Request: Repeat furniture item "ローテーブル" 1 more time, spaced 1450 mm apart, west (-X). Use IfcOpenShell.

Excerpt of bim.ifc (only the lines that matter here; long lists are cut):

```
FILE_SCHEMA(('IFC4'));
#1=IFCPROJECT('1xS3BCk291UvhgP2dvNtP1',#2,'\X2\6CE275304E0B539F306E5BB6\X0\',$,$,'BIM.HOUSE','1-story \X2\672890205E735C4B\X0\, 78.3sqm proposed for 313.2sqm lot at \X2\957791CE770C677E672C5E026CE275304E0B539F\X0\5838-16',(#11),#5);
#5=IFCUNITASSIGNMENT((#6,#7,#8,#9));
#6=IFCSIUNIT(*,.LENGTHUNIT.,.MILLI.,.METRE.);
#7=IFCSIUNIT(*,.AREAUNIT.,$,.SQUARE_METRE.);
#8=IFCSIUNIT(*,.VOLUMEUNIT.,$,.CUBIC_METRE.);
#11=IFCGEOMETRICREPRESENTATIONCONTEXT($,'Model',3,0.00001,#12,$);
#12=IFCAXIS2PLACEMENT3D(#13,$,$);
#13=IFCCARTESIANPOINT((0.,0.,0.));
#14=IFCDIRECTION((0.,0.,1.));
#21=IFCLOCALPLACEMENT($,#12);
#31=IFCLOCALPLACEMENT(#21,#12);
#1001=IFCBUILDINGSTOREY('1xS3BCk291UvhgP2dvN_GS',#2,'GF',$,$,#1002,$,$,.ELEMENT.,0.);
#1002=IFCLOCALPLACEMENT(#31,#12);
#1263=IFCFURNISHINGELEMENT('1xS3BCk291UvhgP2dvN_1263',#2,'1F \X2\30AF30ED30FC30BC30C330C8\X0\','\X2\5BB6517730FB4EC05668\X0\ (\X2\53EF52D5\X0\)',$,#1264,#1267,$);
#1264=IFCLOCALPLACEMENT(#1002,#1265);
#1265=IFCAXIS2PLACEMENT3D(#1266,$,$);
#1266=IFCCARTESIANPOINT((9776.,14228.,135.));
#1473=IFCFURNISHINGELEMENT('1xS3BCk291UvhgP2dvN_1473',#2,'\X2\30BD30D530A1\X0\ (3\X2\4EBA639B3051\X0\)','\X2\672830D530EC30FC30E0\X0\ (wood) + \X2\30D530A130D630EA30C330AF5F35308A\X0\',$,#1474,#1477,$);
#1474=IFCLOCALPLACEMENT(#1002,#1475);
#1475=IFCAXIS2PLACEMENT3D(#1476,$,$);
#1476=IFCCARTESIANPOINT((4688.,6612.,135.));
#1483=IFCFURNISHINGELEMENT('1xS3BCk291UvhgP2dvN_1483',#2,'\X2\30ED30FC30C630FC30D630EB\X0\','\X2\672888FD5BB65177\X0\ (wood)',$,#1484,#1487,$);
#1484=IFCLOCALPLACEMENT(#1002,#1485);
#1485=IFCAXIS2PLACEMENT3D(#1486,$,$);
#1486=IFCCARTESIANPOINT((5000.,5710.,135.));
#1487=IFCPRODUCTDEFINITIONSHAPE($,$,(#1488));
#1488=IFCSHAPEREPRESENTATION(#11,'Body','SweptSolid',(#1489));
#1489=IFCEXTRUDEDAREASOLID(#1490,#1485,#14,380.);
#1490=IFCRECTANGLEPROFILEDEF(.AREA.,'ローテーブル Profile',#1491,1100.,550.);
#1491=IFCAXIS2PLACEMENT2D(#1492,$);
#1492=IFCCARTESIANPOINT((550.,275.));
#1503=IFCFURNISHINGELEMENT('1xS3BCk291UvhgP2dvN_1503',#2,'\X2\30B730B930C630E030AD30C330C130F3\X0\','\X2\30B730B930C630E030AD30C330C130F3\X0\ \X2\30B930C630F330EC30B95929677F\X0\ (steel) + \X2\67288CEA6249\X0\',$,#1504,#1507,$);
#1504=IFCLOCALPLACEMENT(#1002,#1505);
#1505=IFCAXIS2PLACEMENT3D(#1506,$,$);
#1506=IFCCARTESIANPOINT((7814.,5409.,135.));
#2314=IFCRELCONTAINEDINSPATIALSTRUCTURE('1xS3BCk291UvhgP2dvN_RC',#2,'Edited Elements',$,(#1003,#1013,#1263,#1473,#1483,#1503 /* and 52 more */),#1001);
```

```python
import numpy as np
import ifcopenshell
import ifcopenshell.api.geometry
import ifcopenshell.api.root
import ifcopenshell.util.element
import ifcopenshell.util.placement
import ifcopenshell.util.unit

model = ifcopenshell.open("bim.ifc")
unit_scale = ifcopenshell.util.unit.calculate_unit_scale(model)


def reuse_history(source, copy):
    """copy_class also copies each property set's owner history, people and application; keep the originals."""
    for rel in copy.IsDefinedBy:
        if rel.is_a("IfcRelDefinesByProperties") and (history := rel.RelatingPropertyDefinition.OwnerHistory):
            rel.RelatingPropertyDefinition.OwnerHistory = source.OwnerHistory
            ifcopenshell.util.element.remove_deep2(model, history)


source = model.by_guid("1xS3BCk291UvhgP2dvN_1483")
base = ifcopenshell.util.placement.get_local_placement(source.ObjectPlacement)
step = np.array([-1.0, 0.0, 0.0]) * 1.45 / unit_scale

for i in range(1, 2):
    copy = ifcopenshell.api.root.copy_class(model, product=source)
    copy.Representation = ifcopenshell.util.element.copy_deep(
        model, source.Representation, exclude=["IfcGeometricRepresentationContext", "IfcRepresentationMap"]
    )
    reuse_history(source, copy)
    matrix = base.copy()
    matrix[:3, 3] += i * step
    print("added at", matrix[:3, 3].round(3) + 0.0)
    ifcopenshell.api.geometry.edit_object_placement(model, product=copy, matrix=matrix, is_si=False)

model.write("bim_rev.ifc")
```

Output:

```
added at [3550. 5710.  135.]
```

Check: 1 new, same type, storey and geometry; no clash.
